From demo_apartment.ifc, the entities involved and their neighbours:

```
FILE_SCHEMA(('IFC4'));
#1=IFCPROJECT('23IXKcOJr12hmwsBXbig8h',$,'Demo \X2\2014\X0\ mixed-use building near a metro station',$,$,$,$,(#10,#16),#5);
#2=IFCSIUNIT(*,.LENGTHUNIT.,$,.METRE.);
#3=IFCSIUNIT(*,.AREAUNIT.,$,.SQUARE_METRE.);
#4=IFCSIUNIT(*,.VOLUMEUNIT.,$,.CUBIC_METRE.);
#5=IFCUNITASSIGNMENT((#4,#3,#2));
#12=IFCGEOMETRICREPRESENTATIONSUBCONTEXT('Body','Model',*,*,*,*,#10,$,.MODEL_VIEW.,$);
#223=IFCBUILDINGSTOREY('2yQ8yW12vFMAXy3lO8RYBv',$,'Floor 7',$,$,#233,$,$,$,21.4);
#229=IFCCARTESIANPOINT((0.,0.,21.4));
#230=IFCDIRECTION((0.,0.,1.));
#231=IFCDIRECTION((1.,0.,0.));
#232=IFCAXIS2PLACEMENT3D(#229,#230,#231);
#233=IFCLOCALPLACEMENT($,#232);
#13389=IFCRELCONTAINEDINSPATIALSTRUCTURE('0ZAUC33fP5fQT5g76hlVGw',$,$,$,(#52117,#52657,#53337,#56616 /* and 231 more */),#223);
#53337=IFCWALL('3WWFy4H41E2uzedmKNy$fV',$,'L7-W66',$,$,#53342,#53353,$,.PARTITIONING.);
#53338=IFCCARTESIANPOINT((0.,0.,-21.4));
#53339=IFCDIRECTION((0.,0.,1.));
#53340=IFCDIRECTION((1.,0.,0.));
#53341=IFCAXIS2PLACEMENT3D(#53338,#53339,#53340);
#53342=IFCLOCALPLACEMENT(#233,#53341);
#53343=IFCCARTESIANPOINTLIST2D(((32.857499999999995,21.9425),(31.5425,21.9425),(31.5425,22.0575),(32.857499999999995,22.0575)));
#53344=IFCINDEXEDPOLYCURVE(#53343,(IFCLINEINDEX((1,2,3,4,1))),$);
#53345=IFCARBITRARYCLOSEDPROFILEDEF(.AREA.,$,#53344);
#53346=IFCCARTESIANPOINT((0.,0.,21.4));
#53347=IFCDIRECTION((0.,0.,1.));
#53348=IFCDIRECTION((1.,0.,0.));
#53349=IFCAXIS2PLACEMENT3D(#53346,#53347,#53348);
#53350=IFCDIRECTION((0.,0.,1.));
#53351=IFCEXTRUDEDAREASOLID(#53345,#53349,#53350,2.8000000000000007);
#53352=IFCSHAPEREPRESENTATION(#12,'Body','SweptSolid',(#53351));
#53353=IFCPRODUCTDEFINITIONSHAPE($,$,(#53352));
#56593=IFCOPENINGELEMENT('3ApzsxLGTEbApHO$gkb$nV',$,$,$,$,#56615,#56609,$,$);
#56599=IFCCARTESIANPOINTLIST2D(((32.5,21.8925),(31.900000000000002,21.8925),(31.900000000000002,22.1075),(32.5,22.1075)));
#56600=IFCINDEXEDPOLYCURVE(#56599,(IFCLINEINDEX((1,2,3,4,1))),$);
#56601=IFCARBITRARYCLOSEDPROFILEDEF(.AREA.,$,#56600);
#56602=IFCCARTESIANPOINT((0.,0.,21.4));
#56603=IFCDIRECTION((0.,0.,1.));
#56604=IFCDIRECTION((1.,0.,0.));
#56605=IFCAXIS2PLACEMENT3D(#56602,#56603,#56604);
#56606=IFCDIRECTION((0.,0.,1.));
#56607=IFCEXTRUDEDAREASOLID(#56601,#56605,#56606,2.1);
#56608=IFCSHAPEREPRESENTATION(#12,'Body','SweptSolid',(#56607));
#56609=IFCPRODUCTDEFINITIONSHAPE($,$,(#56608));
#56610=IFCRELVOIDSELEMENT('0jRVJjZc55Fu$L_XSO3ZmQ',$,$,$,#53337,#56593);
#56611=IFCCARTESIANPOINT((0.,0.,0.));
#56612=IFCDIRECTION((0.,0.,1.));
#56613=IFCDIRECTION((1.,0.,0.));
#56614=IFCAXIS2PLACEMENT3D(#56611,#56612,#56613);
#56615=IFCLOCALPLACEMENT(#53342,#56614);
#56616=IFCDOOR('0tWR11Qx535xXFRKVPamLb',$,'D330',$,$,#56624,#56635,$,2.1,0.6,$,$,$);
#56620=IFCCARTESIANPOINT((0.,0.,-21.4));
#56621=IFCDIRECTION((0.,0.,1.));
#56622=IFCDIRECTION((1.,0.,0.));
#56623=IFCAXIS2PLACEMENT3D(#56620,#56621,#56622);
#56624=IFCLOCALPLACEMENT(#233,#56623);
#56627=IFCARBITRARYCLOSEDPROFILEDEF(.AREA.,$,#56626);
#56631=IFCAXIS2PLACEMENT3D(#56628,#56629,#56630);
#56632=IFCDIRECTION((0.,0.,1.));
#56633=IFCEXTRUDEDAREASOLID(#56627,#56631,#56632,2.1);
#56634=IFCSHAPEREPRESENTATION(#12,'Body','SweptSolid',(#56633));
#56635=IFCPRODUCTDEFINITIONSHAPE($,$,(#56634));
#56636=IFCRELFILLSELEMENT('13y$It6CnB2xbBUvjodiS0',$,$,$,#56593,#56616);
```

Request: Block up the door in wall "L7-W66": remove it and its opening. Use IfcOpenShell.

```python
import ifcopenshell
import ifcopenshell.api.feature
import ifcopenshell.api.root
import ifcopenshell.geom
import ifcopenshell.util.shape

model = ifcopenshell.open("demo_apartment.ifc")
settings = ifcopenshell.geom.settings()


def volume(element):
    """Net volume in cubic metres, openings subtracted."""
    shape = ifcopenshell.geom.create_shape(settings, element)
    return ifcopenshell.util.shape.get_volume(shape.geometry)


door = model.by_id(56616)
opening = door.FillsVoids[0].RelatingOpeningElement
wall = opening.VoidsElements[0].RelatingBuildingElement
before = volume(wall)

ifcopenshell.api.root.remove_product(model, product=door)
ifcopenshell.api.feature.remove_feature(model, feature=opening)

after = volume(wall)

print(f"wall volume {before:.3f} -> {after:.3f} m3")

model.write("demo_apartment_edited.ifc")
```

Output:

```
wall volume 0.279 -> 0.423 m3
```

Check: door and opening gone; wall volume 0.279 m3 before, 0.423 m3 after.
